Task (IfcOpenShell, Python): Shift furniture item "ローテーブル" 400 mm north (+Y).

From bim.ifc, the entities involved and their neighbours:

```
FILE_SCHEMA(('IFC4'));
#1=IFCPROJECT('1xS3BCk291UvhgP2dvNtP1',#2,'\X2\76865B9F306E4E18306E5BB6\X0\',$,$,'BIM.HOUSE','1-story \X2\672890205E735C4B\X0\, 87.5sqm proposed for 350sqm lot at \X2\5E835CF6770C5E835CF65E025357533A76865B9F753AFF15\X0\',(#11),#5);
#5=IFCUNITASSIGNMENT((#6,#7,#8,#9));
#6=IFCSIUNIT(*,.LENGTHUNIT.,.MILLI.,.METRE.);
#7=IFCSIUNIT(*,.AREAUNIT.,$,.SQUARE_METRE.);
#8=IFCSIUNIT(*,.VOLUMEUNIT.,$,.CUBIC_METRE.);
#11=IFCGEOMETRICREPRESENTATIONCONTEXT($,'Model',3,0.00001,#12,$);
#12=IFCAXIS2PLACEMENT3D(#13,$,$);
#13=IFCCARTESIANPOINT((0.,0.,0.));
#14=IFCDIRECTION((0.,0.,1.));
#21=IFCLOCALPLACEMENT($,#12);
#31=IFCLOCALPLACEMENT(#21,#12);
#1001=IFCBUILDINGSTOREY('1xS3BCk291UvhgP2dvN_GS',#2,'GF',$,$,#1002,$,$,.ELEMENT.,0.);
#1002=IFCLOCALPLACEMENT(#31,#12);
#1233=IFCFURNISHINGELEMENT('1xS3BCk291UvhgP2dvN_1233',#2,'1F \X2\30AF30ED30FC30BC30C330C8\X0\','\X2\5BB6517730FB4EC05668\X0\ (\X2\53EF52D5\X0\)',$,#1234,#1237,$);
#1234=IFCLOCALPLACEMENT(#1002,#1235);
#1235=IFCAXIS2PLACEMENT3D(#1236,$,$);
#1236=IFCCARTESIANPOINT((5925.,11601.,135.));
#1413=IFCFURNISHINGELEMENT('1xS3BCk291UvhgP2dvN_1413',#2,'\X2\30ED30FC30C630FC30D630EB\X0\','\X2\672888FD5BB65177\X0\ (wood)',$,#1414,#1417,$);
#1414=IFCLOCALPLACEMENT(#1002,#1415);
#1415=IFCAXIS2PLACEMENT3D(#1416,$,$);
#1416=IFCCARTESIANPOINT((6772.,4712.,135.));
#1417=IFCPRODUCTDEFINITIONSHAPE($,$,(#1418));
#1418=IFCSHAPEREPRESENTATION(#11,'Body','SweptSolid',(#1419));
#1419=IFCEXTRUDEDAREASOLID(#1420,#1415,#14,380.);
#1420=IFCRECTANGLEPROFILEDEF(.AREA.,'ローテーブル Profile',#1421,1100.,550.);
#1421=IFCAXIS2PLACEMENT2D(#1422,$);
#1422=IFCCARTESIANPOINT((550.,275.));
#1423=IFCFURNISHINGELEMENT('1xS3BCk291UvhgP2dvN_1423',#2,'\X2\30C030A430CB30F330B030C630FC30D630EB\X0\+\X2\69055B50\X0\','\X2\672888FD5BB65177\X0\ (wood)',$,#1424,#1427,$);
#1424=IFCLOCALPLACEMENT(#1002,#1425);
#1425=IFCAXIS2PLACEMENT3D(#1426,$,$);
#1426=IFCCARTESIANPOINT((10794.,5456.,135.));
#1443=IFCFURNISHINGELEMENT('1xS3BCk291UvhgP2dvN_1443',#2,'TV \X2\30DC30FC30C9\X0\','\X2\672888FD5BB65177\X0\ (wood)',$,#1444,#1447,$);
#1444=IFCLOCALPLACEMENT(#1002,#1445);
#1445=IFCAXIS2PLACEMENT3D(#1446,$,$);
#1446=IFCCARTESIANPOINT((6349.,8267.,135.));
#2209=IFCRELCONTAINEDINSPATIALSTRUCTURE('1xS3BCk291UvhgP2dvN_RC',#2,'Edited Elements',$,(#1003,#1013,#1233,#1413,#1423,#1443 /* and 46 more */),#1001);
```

```python
import ifcopenshell
import ifcopenshell.api.geometry
import ifcopenshell.util.placement

model = ifcopenshell.open("bim.ifc")

item = model.by_id(1413)
matrix = ifcopenshell.util.placement.get_local_placement(item.ObjectPlacement)
matrix[1, 3] += 400.0
ifcopenshell.api.geometry.edit_object_placement(model, product=item, matrix=matrix, is_si=False)

print(ifcopenshell.util.placement.get_local_placement(item.ObjectPlacement).round(3) + 0.0)

model.write("bim_updated.ifc")
```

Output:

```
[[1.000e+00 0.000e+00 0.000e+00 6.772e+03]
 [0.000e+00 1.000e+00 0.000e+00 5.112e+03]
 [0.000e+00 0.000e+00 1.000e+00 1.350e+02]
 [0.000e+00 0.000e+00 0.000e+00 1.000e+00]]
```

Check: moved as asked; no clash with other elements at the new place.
